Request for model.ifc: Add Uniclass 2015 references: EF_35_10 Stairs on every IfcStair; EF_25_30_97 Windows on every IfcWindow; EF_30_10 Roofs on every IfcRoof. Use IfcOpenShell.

First a look at what the model holds.

```python
import ifcopenshell

model = ifcopenshell.open("model.ifc")
print(model.schema)
print("classifications:", [c.Name for c in model.by_type("IfcClassification")])
for ifc_class in ("IfcDoor", "IfcRoof", "IfcStair", "IfcWall", "IfcWindow"):
    print(ifc_class, len(model.by_type(ifc_class)))
```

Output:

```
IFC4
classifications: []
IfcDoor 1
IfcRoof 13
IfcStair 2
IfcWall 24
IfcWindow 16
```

```python
import ifcopenshell
import ifcopenshell.api.classification

model = ifcopenshell.open("model.ifc")

system = ifcopenshell.api.classification.add_classification(model, classification="Uniclass 2015")

codes = {
    "IfcStair": ("EF_35_10", "Stairs"),
    "IfcWindow": ("EF_25_30_97", "Windows"),
    "IfcRoof": ("EF_30_10", "Roofs"),
}
for ifc_class, (code, name) in codes.items():
    products = model.by_type(ifc_class)
    ifcopenshell.api.classification.add_reference(
        model, products=products, classification=system, identification=code, name=name
    )
    print(code, len(products))

model.write("model_v2.ifc")
```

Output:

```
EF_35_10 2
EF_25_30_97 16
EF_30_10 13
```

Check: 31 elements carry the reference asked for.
